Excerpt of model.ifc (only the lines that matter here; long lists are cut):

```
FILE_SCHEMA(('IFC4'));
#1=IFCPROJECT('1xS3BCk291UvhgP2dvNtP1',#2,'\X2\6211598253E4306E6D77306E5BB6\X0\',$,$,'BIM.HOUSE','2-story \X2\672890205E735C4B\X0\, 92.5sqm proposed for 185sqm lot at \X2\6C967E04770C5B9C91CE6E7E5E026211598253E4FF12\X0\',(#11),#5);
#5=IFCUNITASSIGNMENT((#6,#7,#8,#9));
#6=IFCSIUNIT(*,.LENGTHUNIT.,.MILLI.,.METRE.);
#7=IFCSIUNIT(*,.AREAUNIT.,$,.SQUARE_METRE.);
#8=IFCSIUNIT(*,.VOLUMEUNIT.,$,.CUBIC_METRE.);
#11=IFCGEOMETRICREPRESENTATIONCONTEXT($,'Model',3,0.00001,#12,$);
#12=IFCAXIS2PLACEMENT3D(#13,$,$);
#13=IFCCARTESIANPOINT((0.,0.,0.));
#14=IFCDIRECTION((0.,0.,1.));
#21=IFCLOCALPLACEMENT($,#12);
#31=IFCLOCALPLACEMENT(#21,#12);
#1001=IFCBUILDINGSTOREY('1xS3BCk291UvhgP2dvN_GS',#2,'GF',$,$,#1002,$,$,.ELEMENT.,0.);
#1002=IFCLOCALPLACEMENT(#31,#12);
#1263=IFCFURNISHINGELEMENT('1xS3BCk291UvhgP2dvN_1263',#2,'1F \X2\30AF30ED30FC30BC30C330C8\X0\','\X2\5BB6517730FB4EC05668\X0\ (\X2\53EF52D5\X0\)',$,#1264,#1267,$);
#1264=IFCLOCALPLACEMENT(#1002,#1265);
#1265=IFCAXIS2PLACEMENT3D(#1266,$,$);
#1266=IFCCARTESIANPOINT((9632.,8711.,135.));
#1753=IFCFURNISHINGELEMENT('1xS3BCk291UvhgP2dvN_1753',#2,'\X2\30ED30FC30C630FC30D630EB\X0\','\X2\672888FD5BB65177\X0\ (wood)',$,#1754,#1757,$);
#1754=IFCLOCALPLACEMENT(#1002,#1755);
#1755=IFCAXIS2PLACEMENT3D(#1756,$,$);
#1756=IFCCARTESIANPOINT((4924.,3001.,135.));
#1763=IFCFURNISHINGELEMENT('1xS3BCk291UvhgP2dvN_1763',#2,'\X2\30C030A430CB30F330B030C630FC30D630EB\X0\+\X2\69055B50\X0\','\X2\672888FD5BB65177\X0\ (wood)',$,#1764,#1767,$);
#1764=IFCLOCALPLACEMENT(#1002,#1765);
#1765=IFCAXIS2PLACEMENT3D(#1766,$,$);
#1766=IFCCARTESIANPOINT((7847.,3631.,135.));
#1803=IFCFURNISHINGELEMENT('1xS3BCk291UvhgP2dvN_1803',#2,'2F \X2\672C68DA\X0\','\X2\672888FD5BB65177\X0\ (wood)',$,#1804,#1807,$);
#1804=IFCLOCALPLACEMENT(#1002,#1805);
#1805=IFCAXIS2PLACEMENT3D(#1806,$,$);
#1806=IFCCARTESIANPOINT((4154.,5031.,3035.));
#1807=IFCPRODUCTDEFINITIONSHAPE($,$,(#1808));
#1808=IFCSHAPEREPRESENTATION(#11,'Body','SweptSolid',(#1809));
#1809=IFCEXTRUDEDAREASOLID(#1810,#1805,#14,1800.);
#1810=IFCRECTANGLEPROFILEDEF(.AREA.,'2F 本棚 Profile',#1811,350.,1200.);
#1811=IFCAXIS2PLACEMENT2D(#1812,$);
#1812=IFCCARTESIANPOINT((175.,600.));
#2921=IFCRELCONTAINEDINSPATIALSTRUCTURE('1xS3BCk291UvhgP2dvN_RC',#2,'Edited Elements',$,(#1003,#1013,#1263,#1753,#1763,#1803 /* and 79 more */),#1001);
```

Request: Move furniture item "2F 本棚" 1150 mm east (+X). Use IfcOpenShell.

```python
import ifcopenshell
import ifcopenshell.api.geometry
import ifcopenshell.util.placement
import ifcopenshell.util.unit

model = ifcopenshell.open("model.ifc")
unit_scale = ifcopenshell.util.unit.calculate_unit_scale(model)

item = model.by_guid("1xS3BCk291UvhgP2dvN_1803")
matrix = ifcopenshell.util.placement.get_local_placement(item.ObjectPlacement)
matrix[0, 3] += 1.15 / unit_scale
ifcopenshell.api.geometry.edit_object_placement(model, product=item, matrix=matrix, is_si=False)

print(ifcopenshell.util.placement.get_local_placement(item.ObjectPlacement).round(3) + 0.0)

model.write("model_edited.ifc")
```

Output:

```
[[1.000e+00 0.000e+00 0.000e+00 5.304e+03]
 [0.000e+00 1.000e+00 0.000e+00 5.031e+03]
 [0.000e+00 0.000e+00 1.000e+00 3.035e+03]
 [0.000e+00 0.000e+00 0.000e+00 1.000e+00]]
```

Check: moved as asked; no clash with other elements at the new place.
